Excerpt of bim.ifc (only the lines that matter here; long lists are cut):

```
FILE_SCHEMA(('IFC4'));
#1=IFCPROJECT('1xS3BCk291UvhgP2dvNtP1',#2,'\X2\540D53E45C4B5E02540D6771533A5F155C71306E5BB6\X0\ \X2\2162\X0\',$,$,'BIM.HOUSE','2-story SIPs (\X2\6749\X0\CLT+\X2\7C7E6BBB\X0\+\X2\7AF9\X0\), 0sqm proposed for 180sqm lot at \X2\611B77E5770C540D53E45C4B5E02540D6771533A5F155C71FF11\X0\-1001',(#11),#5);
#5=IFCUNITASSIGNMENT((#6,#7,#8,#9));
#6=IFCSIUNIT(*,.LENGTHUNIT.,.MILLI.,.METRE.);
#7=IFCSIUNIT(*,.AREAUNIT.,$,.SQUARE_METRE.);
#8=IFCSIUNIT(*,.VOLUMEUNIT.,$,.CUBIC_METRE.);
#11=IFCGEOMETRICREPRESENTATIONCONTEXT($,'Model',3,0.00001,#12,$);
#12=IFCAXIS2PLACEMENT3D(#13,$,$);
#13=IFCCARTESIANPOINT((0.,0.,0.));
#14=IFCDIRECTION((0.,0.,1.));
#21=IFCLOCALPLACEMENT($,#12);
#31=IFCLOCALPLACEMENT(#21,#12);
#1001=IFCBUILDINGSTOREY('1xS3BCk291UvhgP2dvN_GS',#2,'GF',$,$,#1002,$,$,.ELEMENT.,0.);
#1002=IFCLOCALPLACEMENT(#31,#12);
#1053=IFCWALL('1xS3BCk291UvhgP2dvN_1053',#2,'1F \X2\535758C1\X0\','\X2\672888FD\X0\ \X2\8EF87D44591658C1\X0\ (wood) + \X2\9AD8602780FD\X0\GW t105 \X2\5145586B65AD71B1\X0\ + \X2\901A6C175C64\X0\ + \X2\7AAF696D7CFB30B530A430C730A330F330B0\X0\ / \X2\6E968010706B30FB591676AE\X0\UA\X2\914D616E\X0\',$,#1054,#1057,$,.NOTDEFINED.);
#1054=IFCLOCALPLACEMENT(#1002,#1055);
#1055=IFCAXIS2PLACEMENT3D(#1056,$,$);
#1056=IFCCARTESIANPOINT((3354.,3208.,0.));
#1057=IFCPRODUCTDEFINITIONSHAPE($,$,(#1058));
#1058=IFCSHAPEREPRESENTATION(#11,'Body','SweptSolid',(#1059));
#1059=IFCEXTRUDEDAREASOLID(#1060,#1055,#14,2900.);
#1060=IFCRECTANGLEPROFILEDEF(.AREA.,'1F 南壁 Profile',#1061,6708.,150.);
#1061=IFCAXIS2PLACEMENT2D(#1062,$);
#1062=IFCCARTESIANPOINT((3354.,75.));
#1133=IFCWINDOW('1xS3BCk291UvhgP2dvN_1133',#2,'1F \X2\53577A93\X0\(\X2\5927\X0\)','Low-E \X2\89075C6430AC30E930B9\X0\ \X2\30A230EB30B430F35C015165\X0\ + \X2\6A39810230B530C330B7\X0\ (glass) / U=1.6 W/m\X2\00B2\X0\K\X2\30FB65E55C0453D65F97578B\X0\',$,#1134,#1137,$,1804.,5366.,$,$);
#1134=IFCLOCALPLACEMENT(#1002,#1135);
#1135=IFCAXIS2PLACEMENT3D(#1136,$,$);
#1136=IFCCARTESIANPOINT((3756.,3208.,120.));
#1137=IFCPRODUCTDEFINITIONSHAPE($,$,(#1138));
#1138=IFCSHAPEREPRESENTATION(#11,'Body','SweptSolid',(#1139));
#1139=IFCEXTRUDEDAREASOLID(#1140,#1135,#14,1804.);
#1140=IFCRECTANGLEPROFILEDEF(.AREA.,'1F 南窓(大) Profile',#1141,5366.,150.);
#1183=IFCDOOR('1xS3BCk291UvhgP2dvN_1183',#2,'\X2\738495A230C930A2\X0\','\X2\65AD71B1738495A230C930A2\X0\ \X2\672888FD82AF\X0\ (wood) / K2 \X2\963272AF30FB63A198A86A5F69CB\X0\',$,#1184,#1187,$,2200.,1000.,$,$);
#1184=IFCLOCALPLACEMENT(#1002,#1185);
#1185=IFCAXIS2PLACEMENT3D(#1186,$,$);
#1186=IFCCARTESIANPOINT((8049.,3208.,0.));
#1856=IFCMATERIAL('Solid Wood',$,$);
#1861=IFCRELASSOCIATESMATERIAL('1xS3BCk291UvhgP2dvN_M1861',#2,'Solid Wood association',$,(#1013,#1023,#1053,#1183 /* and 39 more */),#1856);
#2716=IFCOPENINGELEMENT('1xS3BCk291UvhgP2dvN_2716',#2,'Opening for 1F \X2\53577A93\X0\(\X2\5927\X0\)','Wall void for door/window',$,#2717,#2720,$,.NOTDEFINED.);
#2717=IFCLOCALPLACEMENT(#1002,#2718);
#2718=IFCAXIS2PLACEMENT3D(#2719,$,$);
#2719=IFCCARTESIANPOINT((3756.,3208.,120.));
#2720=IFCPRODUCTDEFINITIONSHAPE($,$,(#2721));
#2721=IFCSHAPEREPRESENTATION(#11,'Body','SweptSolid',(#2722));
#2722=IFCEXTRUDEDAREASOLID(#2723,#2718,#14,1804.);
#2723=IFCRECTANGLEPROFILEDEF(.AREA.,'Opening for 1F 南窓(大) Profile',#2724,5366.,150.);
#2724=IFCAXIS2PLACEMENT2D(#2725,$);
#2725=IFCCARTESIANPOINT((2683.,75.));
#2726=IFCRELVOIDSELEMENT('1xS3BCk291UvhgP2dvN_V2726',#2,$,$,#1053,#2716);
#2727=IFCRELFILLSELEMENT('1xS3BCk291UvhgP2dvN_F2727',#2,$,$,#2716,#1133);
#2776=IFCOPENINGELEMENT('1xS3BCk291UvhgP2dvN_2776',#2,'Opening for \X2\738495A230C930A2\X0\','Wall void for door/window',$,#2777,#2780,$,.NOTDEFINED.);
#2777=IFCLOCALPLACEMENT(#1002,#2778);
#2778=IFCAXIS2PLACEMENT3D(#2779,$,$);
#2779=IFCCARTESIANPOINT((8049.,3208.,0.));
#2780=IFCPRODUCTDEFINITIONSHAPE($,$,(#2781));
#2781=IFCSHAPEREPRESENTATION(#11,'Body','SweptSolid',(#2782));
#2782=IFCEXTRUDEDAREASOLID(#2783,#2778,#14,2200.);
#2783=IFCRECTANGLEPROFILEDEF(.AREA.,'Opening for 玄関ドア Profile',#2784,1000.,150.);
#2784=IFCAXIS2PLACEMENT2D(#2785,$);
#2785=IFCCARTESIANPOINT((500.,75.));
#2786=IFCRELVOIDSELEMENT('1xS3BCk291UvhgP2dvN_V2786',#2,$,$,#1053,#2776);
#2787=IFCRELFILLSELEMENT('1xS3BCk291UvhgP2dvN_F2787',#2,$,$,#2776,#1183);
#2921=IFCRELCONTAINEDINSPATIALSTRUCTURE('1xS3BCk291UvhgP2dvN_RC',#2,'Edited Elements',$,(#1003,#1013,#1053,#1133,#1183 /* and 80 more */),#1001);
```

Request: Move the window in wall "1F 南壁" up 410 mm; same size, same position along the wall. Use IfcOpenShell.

```python
import numpy as np
import ifcopenshell
import ifcopenshell.api.geometry
import ifcopenshell.util.placement
import ifcopenshell.util.unit

model = ifcopenshell.open("bim.ifc")
unit_scale = ifcopenshell.util.unit.calculate_unit_scale(model)

window = model.by_id(1133)
opening = window.FillsVoids[0].RelatingOpeningElement
dz = 0.41 / unit_scale

shift = np.array([0.0, 0.0, dz])
# The window is not placed relative to its opening, so move both.
for product in (opening, window):
    matrix = ifcopenshell.util.placement.get_local_placement(product.ObjectPlacement)
    matrix[:3, 3] += shift
    ifcopenshell.api.geometry.edit_object_placement(model, product=product, matrix=matrix, is_si=False)

print(f"moved by {dz * unit_scale:+.3f} m")

model.write("bim_rev.ifc")
```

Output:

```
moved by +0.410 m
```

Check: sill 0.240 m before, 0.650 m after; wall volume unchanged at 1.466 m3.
